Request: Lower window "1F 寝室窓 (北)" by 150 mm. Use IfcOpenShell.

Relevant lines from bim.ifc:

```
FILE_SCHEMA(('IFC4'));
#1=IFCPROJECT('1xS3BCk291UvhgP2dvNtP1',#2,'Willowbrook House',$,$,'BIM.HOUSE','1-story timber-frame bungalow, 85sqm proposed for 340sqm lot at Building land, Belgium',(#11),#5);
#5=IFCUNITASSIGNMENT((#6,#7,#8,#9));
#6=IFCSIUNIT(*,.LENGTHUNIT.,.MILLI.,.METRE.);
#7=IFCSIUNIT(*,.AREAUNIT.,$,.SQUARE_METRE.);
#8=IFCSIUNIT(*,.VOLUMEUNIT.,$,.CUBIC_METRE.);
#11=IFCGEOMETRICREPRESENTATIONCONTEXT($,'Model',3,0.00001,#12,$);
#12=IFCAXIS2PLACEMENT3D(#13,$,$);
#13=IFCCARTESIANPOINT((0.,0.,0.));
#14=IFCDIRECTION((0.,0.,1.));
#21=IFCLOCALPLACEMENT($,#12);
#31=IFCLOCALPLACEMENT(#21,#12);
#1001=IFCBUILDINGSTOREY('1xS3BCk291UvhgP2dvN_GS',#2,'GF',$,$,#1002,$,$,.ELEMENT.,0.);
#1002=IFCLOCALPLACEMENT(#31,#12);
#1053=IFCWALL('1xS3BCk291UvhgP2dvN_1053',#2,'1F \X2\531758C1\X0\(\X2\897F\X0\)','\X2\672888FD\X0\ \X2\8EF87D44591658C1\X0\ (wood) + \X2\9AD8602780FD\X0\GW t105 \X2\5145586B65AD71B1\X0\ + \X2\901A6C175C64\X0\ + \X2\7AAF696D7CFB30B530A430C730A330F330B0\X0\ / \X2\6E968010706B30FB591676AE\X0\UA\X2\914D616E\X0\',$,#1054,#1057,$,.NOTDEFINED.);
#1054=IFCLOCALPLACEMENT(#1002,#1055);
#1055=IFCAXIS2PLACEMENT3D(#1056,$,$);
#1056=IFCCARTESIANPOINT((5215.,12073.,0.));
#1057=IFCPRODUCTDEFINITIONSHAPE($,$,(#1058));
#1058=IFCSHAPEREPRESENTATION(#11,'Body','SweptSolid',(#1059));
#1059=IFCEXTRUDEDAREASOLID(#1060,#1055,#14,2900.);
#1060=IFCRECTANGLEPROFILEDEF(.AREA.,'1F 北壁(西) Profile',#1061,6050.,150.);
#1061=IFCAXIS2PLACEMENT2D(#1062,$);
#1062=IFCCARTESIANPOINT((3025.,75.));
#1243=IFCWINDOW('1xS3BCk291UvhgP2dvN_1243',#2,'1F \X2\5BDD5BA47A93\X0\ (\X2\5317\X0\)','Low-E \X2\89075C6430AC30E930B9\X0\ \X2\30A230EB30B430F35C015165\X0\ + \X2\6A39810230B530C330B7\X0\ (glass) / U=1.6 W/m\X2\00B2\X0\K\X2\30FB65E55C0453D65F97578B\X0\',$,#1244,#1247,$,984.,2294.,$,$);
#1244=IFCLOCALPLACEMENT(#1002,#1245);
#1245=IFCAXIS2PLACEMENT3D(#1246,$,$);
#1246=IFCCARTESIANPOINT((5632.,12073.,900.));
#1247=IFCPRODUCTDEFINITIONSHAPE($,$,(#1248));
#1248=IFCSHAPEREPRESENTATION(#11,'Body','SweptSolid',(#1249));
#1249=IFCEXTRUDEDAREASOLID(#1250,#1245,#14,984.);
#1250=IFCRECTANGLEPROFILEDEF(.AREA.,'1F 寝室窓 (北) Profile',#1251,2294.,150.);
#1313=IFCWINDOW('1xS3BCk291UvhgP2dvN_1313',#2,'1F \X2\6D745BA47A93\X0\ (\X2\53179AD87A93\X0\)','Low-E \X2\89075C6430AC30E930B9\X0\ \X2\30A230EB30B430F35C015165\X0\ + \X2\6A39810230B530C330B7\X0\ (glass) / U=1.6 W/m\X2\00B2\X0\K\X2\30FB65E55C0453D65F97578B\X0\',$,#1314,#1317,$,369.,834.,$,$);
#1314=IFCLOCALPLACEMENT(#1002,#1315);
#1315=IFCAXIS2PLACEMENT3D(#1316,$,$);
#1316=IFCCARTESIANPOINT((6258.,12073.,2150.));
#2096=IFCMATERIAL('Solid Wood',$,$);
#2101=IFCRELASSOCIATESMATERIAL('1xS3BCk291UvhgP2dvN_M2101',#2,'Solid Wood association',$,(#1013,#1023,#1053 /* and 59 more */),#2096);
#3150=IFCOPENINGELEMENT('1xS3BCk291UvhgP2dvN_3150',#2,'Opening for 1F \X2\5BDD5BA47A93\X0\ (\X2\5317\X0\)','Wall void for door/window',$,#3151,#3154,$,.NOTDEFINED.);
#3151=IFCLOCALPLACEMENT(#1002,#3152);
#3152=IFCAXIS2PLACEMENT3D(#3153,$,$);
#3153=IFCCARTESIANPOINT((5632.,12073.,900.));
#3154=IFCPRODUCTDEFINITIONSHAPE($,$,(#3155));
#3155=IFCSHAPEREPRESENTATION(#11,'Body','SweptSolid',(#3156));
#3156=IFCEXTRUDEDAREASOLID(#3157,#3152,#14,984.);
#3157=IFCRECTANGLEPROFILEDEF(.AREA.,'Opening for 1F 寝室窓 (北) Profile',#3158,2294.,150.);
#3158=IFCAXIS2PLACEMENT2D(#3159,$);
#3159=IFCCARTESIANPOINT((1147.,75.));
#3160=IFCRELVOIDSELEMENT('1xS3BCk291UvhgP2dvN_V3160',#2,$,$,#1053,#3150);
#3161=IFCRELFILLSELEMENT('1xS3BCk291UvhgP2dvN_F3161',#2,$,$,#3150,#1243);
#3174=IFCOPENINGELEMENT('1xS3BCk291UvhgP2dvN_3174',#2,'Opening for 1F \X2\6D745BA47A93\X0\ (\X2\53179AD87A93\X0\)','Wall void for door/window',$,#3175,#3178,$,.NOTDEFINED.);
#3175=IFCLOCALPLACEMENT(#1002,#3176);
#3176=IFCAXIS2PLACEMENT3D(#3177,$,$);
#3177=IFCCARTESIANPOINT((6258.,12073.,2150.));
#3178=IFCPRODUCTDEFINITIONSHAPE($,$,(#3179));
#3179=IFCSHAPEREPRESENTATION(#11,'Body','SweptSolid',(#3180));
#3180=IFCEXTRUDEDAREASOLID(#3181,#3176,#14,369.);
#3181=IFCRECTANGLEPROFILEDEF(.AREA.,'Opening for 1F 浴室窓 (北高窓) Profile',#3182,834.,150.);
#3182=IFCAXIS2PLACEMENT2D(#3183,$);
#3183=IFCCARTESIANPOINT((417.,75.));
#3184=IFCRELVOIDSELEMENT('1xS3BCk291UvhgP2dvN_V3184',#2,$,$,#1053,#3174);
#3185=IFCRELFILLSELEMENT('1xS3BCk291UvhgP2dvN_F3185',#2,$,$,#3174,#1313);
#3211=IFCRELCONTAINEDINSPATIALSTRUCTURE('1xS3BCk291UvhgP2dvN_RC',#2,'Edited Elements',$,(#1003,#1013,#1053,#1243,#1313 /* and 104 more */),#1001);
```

```python
import numpy as np
import ifcopenshell
import ifcopenshell.api.geometry
import ifcopenshell.util.placement
import ifcopenshell.util.unit

model = ifcopenshell.open("bim.ifc")
unit_scale = ifcopenshell.util.unit.calculate_unit_scale(model)

window = model.by_guid("1xS3BCk291UvhgP2dvN_1243")
opening = window.FillsVoids[0].RelatingOpeningElement
dz = -150.0

shift = np.array([0.0, 0.0, dz])
# The window is not placed relative to its opening, so move both.
for product in (opening, window):
    matrix = ifcopenshell.util.placement.get_local_placement(product.ObjectPlacement)
    matrix[:3, 3] += shift
    ifcopenshell.api.geometry.edit_object_placement(model, product=product, matrix=matrix, is_si=False)

print(f"moved by {dz * unit_scale:+.3f} m")

model.write("bim_updated.ifc")
```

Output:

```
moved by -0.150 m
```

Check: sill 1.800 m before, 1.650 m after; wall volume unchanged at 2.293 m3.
